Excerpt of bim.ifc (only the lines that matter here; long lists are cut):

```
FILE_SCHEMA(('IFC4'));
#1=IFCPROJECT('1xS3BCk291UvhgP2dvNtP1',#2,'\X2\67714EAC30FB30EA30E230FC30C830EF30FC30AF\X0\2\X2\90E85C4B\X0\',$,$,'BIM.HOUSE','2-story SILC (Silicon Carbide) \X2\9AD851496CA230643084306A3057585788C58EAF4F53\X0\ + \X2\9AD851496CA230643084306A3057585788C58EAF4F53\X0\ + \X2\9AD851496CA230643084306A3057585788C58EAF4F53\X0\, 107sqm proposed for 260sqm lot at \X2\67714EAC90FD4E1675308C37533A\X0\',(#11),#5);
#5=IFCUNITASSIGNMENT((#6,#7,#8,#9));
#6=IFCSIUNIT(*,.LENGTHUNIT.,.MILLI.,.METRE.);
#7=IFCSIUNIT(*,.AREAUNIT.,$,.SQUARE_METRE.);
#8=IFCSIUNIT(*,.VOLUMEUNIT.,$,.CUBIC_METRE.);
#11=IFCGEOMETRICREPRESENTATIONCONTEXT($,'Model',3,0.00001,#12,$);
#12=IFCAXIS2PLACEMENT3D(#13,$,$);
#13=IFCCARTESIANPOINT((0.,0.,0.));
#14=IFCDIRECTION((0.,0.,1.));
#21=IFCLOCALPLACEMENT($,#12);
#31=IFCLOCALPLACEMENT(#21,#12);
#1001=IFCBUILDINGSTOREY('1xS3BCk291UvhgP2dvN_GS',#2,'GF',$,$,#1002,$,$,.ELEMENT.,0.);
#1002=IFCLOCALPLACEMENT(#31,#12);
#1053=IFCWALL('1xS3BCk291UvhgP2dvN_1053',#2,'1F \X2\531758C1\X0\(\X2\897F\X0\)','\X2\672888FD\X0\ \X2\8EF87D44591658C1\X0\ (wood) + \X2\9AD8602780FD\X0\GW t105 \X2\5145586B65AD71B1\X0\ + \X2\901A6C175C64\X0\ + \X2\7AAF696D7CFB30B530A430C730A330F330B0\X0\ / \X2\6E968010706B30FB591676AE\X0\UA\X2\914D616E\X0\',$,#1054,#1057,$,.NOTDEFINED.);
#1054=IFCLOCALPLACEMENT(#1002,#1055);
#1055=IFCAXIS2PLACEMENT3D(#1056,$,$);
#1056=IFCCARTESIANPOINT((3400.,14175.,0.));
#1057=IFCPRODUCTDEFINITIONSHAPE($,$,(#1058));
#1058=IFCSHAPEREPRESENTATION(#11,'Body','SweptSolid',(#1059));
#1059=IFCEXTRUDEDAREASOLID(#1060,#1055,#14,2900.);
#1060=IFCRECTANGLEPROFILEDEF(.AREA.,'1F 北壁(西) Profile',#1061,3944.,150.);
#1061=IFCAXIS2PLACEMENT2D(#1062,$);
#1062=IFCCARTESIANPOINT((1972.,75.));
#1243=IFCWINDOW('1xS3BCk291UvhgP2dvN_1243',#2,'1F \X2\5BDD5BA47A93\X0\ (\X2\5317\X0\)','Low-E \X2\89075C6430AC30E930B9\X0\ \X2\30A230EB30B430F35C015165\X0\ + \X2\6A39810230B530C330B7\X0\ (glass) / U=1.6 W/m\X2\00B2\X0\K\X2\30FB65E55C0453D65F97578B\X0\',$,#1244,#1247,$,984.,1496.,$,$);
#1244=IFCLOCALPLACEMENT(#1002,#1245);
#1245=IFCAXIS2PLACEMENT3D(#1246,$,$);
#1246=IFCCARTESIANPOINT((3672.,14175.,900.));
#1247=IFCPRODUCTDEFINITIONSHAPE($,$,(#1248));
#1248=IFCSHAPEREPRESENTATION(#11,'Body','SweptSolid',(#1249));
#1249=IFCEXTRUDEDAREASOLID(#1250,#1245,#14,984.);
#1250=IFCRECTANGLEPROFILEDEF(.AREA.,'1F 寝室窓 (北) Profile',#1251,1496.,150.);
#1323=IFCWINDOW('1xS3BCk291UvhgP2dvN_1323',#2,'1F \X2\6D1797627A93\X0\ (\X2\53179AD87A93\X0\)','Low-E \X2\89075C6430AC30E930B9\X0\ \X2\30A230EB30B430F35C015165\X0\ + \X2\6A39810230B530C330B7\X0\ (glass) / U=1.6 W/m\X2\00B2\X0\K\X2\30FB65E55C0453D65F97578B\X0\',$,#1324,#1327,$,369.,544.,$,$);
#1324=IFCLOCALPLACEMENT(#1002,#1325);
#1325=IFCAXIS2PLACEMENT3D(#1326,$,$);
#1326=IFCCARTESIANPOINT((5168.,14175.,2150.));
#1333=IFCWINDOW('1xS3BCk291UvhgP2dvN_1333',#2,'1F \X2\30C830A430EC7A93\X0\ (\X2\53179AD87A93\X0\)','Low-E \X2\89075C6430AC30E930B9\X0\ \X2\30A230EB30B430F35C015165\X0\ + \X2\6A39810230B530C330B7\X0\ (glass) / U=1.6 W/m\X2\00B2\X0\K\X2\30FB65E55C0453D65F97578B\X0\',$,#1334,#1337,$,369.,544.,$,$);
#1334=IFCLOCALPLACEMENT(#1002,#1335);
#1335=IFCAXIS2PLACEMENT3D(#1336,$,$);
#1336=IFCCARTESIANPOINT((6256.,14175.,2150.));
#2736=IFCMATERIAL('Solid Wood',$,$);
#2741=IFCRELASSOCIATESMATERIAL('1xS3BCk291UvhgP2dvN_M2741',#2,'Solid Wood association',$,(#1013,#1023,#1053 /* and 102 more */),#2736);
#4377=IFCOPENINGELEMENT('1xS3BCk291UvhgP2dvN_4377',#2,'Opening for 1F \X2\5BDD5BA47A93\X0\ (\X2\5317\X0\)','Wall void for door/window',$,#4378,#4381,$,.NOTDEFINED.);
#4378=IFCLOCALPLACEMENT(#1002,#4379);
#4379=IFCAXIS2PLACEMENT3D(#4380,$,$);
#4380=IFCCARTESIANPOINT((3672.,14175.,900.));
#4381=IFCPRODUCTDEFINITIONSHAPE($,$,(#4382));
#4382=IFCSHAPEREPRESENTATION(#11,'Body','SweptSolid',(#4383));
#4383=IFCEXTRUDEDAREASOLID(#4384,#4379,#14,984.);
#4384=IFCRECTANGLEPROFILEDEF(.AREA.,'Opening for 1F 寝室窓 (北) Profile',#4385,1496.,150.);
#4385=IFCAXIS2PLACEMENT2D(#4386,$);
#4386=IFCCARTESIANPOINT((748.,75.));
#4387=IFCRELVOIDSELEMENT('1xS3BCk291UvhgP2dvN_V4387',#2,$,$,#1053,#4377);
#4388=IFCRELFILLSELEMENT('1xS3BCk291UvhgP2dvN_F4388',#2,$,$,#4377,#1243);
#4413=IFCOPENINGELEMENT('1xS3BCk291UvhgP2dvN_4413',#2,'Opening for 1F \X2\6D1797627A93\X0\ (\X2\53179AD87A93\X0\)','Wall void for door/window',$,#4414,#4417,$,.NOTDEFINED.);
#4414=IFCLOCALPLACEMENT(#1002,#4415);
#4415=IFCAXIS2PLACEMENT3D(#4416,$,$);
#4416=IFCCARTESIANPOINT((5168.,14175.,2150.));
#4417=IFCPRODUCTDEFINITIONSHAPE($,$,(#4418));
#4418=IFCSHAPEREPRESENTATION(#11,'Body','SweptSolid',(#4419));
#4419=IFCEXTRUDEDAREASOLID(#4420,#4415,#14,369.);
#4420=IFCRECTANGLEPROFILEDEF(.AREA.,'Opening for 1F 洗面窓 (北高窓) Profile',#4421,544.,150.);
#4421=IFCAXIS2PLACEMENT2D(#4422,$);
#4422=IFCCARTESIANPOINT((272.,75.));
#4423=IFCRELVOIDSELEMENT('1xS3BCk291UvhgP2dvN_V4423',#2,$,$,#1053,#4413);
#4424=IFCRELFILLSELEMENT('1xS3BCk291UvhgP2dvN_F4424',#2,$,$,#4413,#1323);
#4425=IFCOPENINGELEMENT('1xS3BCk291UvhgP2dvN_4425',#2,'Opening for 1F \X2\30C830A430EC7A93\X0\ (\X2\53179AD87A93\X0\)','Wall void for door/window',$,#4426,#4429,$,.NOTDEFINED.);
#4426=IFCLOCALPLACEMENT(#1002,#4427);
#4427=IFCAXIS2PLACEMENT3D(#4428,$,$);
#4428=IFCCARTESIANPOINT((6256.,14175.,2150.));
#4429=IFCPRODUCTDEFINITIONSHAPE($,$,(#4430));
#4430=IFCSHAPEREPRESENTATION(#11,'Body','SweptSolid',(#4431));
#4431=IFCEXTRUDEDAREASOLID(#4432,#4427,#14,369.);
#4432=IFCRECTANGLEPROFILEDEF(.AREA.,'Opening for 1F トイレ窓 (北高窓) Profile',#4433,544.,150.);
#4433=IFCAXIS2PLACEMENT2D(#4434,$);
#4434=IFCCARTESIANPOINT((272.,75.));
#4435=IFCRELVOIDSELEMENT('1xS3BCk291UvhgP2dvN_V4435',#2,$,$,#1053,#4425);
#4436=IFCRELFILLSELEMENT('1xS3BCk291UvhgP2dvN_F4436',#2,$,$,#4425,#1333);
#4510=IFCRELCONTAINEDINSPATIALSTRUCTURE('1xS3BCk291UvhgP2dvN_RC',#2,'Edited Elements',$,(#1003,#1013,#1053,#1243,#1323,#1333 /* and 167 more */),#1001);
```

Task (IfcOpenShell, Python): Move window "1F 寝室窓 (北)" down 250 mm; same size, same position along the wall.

```python
import numpy as np
import ifcopenshell
import ifcopenshell.api.geometry
import ifcopenshell.util.placement
import ifcopenshell.util.unit

model = ifcopenshell.open("bim.ifc")
unit_scale = ifcopenshell.util.unit.calculate_unit_scale(model)

window = model.by_guid("1xS3BCk291UvhgP2dvN_1243")
opening = window.FillsVoids[0].RelatingOpeningElement
dz = -0.25 / unit_scale

shift = np.array([0.0, 0.0, dz])
# The window is not placed relative to its opening, so move both.
for product in (opening, window):
    matrix = ifcopenshell.util.placement.get_local_placement(product.ObjectPlacement)
    matrix[:3, 3] += shift
    ifcopenshell.api.geometry.edit_object_placement(model, product=product, matrix=matrix, is_si=False)

print(f"moved by {dz * unit_scale:+.3f} m")

model.write("bim_edited.ifc")
```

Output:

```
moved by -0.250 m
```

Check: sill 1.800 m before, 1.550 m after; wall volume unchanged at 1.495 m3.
